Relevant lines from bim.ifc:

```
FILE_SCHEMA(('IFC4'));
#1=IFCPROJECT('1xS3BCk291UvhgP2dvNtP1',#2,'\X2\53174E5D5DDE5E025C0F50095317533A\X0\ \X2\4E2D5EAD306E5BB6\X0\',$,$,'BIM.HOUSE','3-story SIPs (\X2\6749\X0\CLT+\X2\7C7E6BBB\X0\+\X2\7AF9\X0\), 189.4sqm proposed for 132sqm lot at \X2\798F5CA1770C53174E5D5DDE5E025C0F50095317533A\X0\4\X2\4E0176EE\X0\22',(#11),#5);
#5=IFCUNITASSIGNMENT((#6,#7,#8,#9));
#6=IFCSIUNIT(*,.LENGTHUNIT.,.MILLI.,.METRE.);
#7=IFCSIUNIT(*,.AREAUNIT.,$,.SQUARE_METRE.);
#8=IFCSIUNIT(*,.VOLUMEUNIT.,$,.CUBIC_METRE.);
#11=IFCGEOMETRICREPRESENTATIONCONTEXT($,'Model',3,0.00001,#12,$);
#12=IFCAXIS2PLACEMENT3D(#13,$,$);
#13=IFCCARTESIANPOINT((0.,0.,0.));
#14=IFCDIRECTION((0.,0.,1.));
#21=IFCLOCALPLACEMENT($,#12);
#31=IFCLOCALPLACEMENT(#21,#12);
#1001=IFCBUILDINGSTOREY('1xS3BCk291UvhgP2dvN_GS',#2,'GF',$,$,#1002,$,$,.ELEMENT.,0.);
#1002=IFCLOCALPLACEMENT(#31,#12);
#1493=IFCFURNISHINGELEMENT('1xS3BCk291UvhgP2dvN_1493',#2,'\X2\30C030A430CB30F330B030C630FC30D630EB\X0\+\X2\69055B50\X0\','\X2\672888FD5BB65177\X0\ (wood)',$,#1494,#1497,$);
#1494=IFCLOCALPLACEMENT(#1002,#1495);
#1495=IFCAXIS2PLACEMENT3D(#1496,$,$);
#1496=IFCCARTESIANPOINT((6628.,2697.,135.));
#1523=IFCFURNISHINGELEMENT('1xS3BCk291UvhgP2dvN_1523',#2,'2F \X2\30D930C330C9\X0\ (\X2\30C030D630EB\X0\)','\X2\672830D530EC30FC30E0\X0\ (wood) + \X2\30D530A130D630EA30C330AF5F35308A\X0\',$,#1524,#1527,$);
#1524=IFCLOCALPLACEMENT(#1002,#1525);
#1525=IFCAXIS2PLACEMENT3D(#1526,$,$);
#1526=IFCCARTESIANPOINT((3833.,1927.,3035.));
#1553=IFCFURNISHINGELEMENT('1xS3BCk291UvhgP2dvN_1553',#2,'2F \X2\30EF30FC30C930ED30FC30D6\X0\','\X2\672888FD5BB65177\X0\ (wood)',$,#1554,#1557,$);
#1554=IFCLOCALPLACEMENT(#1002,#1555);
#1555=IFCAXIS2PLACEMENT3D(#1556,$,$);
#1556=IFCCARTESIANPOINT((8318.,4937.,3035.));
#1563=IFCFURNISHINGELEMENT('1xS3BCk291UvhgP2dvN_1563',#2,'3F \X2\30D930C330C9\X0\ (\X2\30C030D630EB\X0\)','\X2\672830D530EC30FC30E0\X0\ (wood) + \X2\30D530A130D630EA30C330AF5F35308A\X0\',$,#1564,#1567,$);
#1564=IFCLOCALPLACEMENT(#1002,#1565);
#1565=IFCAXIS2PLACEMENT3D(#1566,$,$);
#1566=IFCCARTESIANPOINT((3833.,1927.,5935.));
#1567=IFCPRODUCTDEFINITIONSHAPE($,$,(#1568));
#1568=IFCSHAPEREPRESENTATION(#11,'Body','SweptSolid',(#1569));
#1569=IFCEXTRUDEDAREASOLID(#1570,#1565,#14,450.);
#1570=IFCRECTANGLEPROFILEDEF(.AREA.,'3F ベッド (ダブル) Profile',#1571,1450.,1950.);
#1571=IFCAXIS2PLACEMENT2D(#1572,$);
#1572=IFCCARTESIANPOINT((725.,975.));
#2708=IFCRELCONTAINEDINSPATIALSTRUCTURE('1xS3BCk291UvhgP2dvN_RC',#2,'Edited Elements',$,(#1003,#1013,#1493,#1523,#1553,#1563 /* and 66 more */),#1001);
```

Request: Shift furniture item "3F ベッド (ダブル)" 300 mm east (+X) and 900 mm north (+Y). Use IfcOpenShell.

```python
import ifcopenshell
import ifcopenshell.api.geometry
import ifcopenshell.util.placement

model = ifcopenshell.open("bim.ifc")

item = model.by_guid("1xS3BCk291UvhgP2dvN_1563")
matrix = ifcopenshell.util.placement.get_local_placement(item.ObjectPlacement)
matrix[0, 3] += 300.0
matrix[1, 3] += 900.0
ifcopenshell.api.geometry.edit_object_placement(model, product=item, matrix=matrix, is_si=False)

print(ifcopenshell.util.placement.get_local_placement(item.ObjectPlacement).round(3) + 0.0)

model.write("bim_rev.ifc")
```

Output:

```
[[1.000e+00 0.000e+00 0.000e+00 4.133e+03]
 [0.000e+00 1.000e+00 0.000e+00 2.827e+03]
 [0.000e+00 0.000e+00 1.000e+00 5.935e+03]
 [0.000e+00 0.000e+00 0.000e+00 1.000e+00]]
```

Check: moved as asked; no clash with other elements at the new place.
